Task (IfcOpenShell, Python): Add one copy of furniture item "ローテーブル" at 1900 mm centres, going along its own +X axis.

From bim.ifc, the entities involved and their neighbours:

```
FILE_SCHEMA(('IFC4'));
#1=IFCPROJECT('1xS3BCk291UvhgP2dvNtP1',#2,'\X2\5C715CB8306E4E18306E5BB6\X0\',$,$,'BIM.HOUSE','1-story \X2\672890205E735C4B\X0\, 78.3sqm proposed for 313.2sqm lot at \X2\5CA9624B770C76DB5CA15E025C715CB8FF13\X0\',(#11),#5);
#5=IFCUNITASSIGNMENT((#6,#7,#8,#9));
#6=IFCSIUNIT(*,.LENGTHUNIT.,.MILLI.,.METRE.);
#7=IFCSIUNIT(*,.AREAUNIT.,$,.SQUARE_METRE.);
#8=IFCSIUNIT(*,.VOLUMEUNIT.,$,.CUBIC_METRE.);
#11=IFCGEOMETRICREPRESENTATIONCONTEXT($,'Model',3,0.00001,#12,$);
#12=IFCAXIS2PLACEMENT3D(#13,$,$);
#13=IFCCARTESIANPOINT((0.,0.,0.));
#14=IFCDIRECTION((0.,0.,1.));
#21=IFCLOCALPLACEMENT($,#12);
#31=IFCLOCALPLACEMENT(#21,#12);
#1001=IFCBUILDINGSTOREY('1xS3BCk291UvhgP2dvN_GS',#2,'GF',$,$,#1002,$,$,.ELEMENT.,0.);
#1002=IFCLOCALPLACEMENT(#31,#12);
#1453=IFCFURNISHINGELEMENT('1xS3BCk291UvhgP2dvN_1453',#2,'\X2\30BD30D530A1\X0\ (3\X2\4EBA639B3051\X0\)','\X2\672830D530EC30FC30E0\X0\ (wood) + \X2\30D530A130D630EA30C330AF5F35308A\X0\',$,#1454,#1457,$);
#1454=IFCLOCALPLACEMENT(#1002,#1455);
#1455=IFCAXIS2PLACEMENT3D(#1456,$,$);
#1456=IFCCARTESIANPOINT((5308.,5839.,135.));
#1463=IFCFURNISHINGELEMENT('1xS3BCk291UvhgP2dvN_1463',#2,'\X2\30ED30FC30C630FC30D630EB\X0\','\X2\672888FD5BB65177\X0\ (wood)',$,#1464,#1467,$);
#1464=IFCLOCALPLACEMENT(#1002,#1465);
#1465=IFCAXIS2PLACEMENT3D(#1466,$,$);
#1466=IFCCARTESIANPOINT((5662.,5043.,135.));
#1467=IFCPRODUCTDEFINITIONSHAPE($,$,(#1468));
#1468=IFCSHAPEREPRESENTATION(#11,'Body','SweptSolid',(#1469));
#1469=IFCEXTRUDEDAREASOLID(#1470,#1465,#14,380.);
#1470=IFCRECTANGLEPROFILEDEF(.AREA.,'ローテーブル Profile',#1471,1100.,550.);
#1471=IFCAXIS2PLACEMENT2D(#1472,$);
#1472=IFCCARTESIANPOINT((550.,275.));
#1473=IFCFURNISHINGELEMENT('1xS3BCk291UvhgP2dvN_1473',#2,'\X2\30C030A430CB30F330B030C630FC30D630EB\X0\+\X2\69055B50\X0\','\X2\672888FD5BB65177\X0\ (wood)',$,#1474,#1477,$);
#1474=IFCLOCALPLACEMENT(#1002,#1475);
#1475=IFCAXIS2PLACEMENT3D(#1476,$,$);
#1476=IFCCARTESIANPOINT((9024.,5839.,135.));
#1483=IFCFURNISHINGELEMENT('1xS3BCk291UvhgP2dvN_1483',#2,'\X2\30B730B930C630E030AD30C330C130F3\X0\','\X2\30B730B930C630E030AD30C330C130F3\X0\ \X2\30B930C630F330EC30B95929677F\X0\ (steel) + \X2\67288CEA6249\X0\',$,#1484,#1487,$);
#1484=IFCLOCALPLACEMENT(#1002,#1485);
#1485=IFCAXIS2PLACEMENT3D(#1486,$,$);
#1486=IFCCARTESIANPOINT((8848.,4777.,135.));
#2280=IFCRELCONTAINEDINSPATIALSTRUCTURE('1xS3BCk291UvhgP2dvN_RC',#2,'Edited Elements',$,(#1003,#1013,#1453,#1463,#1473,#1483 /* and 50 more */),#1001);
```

```python
import ifcopenshell
import ifcopenshell.api.geometry
import ifcopenshell.api.root
import ifcopenshell.util.element
import ifcopenshell.util.placement
import ifcopenshell.util.unit

model = ifcopenshell.open("bim.ifc")
unit_scale = ifcopenshell.util.unit.calculate_unit_scale(model)


def reuse_history(source, copy):
    """copy_class also copies each property set's owner history, people and application; keep the originals."""
    for rel in copy.IsDefinedBy:
        if rel.is_a("IfcRelDefinesByProperties") and (history := rel.RelatingPropertyDefinition.OwnerHistory):
            rel.RelatingPropertyDefinition.OwnerHistory = source.OwnerHistory
            ifcopenshell.util.element.remove_deep2(model, history)


source = model.by_guid("1xS3BCk291UvhgP2dvN_1463")
base = ifcopenshell.util.placement.get_local_placement(source.ObjectPlacement)
step = base[:3, 0] * 1.9 / unit_scale

for i in range(1, 2):
    copy = ifcopenshell.api.root.copy_class(model, product=source)
    copy.Representation = ifcopenshell.util.element.copy_deep(
        model, source.Representation, exclude=["IfcGeometricRepresentationContext", "IfcRepresentationMap"]
    )
    reuse_history(source, copy)
    matrix = base.copy()
    matrix[:3, 3] += i * step
    print("added at", matrix[:3, 3].round(3) + 0.0)
    ifcopenshell.api.geometry.edit_object_placement(model, product=copy, matrix=matrix, is_si=False)

model.write("bim_updated.ifc")
```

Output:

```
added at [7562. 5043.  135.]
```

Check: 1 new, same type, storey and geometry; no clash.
